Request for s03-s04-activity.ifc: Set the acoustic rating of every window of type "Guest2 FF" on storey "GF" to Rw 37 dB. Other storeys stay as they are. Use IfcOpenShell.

First a look at what the model holds.

```python
import ifcopenshell
import ifcopenshell.util.element

model = ifcopenshell.open("s03-s04-activity.ifc")
print(model.schema)
storey = next(s for s in model.by_type("IfcBuildingStorey") if s.Name == "GF")
windows = [e for e in ifcopenshell.util.element.get_decomposition(storey) if e.is_a("IfcWindow")]
seen = {}
for e in windows:
    element_type = ifcopenshell.util.element.get_type(e)
    key = (element_type.Name if element_type != e and element_type else None, ifcopenshell.util.element.get_pset(e, "Pset_WindowCommon", "AcousticRating"))
    seen[key] = seen.get(key, 0) + 1
for (name, value), count in sorted(seen.items(), key=str):
    print(count, "x", name, "|", value)
```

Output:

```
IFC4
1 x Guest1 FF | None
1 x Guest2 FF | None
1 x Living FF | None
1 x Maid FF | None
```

```python
import ifcopenshell
import ifcopenshell.api.pset
import ifcopenshell.util.element

model = ifcopenshell.open("s03-s04-activity.ifc")

storey = next(s for s in model.by_type("IfcBuildingStorey") if s.Name == "GF")
windows = [e for e in ifcopenshell.util.element.get_decomposition(storey) if e.is_a("IfcWindow")]

count = 0
for e in windows:
    element_type = ifcopenshell.util.element.get_type(e)
    if element_type in (None, e) or element_type.Name != "Guest2 FF":
        continue
    # add_pset returns the element's existing set when there is one.
    pset = ifcopenshell.api.pset.add_pset(model, product=e, name="Pset_WindowCommon")
    ifcopenshell.api.pset.edit_pset(model, pset=pset, properties={"AcousticRating": "Rw 37 dB"})
    count += 1

print(count, "windows updated")

model.write("s03-s04-activity_rev.ifc")
```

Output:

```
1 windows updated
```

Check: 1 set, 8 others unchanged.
